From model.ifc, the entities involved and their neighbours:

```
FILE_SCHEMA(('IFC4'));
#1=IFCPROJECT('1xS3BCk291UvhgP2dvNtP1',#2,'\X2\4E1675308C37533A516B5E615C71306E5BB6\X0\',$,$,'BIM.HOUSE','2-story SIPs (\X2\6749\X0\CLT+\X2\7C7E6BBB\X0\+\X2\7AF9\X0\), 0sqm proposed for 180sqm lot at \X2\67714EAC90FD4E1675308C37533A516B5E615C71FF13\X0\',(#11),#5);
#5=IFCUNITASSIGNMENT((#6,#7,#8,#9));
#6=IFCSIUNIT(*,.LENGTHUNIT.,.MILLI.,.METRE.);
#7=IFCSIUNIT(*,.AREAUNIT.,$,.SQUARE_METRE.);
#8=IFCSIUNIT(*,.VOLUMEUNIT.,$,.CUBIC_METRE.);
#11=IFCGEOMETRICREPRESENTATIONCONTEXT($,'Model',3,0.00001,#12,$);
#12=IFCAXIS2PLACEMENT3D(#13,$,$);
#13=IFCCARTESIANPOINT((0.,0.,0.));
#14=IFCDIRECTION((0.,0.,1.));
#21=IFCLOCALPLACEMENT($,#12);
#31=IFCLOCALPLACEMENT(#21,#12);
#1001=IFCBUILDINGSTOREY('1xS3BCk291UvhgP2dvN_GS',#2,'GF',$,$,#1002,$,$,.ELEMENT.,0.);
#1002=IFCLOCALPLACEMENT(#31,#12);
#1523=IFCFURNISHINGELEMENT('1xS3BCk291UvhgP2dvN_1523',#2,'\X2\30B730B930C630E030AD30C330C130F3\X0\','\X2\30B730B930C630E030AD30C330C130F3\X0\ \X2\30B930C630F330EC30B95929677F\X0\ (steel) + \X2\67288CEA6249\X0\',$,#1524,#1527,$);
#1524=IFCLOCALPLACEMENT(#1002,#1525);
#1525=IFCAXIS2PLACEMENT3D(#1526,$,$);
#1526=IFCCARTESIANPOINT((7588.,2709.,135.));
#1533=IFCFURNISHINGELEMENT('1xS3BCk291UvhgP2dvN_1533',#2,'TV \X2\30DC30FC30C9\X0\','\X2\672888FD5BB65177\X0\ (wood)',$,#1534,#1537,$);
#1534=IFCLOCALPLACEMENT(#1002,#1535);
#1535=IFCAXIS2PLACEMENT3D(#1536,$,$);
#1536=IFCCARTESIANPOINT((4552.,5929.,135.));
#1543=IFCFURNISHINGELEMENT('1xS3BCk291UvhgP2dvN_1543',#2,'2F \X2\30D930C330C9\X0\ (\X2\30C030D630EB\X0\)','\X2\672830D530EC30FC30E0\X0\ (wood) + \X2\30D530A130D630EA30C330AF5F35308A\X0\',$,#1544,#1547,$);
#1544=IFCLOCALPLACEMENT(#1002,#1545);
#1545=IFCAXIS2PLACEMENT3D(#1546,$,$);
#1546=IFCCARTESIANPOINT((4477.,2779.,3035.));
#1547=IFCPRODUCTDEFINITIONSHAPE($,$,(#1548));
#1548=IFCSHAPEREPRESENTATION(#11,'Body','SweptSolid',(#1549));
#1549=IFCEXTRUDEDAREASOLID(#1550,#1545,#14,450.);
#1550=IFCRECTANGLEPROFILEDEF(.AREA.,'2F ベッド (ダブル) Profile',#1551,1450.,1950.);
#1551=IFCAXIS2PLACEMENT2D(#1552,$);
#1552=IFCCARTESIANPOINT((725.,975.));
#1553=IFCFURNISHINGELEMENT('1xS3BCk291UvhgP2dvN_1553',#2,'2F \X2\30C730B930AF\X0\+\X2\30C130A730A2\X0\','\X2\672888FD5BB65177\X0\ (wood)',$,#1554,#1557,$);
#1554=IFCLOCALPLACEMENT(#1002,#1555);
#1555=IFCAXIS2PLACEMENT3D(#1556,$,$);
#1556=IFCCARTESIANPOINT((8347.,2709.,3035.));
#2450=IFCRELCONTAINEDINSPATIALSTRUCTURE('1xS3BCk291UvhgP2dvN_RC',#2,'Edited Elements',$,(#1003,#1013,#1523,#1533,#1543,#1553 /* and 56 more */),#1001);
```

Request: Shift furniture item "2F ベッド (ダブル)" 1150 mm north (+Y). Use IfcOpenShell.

```python
import ifcopenshell
import ifcopenshell.api.geometry
import ifcopenshell.util.placement

model = ifcopenshell.open("model.ifc")

item = model.by_id(1543)
matrix = ifcopenshell.util.placement.get_local_placement(item.ObjectPlacement)
matrix[1, 3] += 1150.0
ifcopenshell.api.geometry.edit_object_placement(model, product=item, matrix=matrix, is_si=False)

print(ifcopenshell.util.placement.get_local_placement(item.ObjectPlacement).round(3) + 0.0)

model.write("model_updated.ifc")
```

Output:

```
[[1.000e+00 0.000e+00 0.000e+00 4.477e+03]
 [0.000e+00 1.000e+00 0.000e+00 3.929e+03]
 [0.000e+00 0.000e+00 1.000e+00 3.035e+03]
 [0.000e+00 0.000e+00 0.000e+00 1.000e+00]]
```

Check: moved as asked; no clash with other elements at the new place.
